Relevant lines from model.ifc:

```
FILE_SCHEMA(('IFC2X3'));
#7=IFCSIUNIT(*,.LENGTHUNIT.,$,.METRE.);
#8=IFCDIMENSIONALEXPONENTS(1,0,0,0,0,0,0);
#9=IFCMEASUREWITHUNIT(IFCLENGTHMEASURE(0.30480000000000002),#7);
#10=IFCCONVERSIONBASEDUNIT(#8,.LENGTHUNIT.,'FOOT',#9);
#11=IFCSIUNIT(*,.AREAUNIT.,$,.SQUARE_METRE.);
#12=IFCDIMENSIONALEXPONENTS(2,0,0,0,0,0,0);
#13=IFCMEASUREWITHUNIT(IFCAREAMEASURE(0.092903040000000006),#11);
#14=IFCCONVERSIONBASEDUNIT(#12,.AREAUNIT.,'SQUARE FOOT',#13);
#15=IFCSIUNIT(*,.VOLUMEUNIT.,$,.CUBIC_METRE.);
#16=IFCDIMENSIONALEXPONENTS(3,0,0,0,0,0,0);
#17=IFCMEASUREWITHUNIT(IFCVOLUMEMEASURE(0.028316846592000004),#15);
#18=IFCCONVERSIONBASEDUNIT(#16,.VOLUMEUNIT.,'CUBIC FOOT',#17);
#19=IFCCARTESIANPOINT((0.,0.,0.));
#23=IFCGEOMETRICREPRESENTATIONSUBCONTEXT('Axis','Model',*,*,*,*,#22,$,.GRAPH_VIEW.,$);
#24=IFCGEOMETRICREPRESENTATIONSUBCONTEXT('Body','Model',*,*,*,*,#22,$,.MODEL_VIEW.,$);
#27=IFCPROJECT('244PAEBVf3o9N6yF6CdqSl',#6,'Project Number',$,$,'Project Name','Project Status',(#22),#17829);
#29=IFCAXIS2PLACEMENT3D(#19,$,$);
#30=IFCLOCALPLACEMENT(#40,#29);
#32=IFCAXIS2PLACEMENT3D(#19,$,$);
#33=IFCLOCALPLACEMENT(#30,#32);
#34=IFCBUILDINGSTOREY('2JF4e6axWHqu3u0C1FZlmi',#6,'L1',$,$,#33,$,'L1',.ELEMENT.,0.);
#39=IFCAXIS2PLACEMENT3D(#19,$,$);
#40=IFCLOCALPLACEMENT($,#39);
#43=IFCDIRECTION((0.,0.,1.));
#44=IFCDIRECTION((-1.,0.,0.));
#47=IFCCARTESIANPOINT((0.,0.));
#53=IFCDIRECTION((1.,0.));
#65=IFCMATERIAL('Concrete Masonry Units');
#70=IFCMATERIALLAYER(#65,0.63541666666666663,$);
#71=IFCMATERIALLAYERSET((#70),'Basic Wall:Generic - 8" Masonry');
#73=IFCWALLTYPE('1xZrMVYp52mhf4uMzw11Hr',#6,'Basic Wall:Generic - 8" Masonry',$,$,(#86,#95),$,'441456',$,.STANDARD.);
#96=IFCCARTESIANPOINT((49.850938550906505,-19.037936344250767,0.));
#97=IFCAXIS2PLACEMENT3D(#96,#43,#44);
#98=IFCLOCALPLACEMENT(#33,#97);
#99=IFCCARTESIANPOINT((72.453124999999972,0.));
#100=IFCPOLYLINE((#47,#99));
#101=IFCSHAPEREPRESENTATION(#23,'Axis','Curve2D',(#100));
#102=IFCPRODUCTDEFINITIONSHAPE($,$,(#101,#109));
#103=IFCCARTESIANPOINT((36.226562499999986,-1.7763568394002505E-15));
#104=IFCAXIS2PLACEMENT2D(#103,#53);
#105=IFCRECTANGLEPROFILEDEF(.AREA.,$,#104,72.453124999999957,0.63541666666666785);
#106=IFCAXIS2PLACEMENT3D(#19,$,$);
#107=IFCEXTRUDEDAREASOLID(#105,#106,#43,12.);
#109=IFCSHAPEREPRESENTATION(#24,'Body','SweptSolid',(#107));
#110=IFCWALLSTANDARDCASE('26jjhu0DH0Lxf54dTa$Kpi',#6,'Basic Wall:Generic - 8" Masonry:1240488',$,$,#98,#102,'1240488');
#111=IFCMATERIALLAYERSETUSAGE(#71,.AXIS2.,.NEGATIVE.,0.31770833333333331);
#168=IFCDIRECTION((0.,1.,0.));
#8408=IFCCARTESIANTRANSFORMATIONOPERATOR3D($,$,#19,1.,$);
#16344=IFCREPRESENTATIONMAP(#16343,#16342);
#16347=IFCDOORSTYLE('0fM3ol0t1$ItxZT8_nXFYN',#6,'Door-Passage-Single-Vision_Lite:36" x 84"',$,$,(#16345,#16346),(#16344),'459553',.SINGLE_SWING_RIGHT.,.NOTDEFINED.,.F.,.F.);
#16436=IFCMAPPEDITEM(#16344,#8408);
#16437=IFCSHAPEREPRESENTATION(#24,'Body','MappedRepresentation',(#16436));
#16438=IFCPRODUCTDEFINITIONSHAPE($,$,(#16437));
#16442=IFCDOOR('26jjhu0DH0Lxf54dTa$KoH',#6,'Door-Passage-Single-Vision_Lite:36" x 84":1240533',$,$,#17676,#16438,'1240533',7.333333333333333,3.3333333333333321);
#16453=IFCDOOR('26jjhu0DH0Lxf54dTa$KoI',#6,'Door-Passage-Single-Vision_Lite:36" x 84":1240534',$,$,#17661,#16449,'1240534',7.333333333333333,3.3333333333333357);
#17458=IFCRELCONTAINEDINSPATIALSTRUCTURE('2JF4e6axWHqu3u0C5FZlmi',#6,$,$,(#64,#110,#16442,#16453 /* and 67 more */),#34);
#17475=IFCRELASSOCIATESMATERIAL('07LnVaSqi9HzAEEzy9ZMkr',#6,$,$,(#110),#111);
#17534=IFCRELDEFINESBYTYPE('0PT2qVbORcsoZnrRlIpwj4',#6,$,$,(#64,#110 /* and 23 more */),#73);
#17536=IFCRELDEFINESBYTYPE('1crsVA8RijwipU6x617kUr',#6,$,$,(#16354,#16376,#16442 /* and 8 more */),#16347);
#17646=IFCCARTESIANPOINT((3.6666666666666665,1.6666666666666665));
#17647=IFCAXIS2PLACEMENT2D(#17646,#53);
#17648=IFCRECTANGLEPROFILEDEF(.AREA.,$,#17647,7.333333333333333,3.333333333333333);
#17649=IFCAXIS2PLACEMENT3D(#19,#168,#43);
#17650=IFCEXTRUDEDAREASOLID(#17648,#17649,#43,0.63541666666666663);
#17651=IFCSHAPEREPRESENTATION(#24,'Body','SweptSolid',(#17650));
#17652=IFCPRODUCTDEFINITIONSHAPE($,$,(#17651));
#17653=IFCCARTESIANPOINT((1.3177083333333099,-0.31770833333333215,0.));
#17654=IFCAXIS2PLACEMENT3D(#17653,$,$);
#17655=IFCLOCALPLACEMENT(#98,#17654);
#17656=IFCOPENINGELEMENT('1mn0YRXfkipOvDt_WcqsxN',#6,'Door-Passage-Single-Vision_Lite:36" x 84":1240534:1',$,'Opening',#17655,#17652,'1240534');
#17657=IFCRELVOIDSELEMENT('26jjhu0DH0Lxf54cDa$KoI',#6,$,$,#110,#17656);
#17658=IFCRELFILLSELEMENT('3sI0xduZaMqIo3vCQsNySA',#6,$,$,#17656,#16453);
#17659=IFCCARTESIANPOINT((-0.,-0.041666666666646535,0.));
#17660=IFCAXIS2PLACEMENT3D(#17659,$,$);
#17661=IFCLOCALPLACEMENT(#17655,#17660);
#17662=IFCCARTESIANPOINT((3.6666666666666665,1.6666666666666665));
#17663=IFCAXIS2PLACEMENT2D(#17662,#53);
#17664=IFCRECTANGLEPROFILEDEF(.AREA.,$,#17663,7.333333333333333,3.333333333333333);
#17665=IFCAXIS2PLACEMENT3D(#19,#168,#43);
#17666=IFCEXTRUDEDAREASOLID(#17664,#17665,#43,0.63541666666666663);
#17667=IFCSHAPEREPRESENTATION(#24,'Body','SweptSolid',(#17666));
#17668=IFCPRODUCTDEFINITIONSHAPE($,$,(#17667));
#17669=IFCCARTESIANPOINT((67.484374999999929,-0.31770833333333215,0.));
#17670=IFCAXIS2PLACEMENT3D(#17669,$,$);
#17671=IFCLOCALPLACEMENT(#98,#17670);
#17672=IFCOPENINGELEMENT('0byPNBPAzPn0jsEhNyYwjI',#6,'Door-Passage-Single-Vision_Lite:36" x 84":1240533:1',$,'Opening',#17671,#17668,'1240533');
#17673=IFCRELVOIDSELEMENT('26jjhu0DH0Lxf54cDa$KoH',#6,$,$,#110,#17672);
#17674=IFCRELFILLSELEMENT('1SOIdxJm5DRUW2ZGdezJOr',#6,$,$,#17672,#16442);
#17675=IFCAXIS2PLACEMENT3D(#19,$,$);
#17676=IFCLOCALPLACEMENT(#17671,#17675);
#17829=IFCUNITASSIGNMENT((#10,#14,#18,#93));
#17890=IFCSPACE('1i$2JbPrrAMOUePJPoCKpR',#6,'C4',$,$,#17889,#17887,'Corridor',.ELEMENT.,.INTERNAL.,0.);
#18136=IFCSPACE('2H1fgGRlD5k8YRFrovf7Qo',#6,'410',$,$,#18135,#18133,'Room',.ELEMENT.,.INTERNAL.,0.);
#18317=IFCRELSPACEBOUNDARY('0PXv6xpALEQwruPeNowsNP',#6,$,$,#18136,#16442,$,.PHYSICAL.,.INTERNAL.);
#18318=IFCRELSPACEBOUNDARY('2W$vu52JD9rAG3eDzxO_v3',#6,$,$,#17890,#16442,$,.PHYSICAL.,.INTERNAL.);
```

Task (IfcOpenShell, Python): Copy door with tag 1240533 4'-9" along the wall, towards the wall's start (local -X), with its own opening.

```python
import ifcopenshell
import ifcopenshell.api.feature
import ifcopenshell.api.geometry
import ifcopenshell.api.root
import ifcopenshell.geom
import ifcopenshell.util.element
import ifcopenshell.util.placement
import ifcopenshell.util.shape
import ifcopenshell.util.unit

model = ifcopenshell.open("model.ifc")
unit_scale = ifcopenshell.util.unit.calculate_unit_scale(model)
settings = ifcopenshell.geom.settings()


def volume(element):
    """Net volume in cubic metres, openings subtracted."""
    shape = ifcopenshell.geom.create_shape(settings, element)
    return ifcopenshell.util.shape.get_volume(shape.geometry)


def reuse_history(source, copy):
    """copy_class also copies each property set's owner history, people and application; keep the originals."""
    for rel in copy.IsDefinedBy:
        if rel.is_a("IfcRelDefinesByProperties") and (history := rel.RelatingPropertyDefinition.OwnerHistory):
            rel.RelatingPropertyDefinition.OwnerHistory = source.OwnerHistory
            ifcopenshell.util.element.remove_deep2(model, history)


door = model.by_guid("26jjhu0DH0Lxf54dTa$KoH")
opening = door.FillsVoids[0].RelatingOpeningElement
wall = opening.VoidsElements[0].RelatingBuildingElement
before = volume(wall)
shift = ifcopenshell.util.placement.get_local_placement(wall.ObjectPlacement)[:3, 0] * -57 * 0.0254 / unit_scale

# copy_class copies the void relationship, type, container and properties, but no geometry.
new_opening = ifcopenshell.api.root.copy_class(model, product=opening)
new_opening.Representation = ifcopenshell.util.element.copy_deep(
    model, opening.Representation, exclude=["IfcGeometricRepresentationContext", "IfcRepresentationMap"]
)
new_opening.Name = 'Door-Passage-Single-Vision_Lite:36" x 84"'
new_opening.Tag = None
new_door = ifcopenshell.api.root.copy_class(model, product=door)
new_door.Representation = ifcopenshell.util.element.copy_deep(
    model, door.Representation, exclude=["IfcGeometricRepresentationContext", "IfcRepresentationMap"]
)
new_door.Name = 'Door-Passage-Single-Vision_Lite:36" x 84"'
new_door.Tag = None
reuse_history(door, new_door)
fills = ifcopenshell.api.feature.add_filling(model, opening=new_opening, element=new_door)
fills.OwnerHistory = new_door.OwnerHistory  # required in IFC2X3

for old, new in ((opening, new_opening), (door, new_door)):
    matrix = ifcopenshell.util.placement.get_local_placement(old.ObjectPlacement)
    matrix[:3, 3] += shift
    ifcopenshell.api.geometry.edit_object_placement(model, product=new, matrix=matrix, is_si=False)

after = volume(wall)

print(f"wall volume {before:.3f} -> {after:.3f} m3")

model.write("model-out.ifc")
```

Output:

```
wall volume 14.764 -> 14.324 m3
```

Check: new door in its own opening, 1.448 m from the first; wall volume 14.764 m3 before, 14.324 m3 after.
